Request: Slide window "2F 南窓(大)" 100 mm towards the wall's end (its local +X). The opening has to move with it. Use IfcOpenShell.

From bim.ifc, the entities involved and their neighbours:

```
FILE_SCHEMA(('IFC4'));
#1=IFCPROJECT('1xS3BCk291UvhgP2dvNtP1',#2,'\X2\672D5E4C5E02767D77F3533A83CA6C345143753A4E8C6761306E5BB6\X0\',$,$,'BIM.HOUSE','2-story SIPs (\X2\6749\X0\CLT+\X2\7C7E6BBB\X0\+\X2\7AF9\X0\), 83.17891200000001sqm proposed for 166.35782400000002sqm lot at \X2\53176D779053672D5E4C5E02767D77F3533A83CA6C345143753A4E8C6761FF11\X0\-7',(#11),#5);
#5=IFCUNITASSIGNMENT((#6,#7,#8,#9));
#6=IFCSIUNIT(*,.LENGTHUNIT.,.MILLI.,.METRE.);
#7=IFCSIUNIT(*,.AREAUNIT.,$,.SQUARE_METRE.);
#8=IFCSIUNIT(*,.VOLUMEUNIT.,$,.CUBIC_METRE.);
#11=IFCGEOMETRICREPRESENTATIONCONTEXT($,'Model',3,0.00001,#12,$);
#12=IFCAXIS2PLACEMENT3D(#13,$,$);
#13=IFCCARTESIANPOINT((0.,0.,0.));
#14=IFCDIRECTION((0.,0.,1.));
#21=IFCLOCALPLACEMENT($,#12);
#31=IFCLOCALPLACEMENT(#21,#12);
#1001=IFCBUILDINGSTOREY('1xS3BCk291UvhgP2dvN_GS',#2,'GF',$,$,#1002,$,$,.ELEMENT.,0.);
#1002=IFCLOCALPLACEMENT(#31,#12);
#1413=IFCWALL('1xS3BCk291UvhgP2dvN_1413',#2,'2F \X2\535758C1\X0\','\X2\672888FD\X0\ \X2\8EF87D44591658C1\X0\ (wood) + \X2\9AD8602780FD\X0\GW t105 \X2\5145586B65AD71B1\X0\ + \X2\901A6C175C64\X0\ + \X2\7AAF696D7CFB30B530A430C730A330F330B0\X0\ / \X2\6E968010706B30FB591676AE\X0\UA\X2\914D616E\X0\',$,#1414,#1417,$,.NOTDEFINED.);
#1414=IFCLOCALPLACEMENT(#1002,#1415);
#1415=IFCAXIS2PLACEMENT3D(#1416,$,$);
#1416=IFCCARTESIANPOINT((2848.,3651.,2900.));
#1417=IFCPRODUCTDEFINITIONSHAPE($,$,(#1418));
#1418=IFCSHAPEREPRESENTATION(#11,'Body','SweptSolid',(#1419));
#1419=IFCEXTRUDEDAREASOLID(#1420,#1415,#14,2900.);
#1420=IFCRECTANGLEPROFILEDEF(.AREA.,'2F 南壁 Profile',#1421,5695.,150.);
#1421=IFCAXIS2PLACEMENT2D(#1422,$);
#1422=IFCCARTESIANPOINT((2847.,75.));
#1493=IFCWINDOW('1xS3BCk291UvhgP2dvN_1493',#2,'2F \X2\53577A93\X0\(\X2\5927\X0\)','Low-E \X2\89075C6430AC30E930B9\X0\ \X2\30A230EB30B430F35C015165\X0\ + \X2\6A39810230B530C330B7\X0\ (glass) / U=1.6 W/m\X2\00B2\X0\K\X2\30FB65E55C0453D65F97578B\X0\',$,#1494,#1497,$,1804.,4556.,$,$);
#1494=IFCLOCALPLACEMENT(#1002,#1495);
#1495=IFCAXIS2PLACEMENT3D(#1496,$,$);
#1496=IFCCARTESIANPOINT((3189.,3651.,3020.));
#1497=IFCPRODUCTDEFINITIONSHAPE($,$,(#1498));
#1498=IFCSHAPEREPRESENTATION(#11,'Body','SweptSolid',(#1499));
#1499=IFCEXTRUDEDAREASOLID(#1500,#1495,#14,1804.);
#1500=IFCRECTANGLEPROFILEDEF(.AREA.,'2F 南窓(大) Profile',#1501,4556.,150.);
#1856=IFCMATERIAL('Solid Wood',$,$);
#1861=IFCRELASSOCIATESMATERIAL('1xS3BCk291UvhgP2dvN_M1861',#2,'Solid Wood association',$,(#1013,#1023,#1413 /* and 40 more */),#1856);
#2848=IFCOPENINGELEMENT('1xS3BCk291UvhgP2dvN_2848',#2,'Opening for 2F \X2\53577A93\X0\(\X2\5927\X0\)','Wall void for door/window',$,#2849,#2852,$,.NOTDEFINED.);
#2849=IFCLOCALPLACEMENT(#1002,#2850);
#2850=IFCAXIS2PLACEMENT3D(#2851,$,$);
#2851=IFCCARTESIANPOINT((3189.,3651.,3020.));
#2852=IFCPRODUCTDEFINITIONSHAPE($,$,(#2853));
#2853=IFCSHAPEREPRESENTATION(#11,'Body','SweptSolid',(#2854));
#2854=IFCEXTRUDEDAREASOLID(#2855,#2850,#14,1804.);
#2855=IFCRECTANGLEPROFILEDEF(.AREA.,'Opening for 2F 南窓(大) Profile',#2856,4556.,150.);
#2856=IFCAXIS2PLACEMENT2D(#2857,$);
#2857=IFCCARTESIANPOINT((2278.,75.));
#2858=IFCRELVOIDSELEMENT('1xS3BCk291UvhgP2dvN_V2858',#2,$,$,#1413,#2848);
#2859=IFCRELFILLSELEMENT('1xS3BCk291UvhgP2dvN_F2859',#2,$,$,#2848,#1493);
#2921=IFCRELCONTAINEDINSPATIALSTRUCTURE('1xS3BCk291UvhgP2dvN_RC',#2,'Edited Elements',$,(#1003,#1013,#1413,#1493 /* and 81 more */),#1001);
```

```python
import ifcopenshell
import ifcopenshell.api.geometry
import ifcopenshell.util.placement
import ifcopenshell.util.unit

model = ifcopenshell.open("bim.ifc")
unit_scale = ifcopenshell.util.unit.calculate_unit_scale(model)

window = model.by_guid("1xS3BCk291UvhgP2dvN_1493")
opening = window.FillsVoids[0].RelatingOpeningElement
wall = opening.VoidsElements[0].RelatingBuildingElement

wall_matrix = ifcopenshell.util.placement.get_local_placement(wall.ObjectPlacement)
shift = wall_matrix[:3, 0] * 0.1 / unit_scale
before = ifcopenshell.util.placement.get_local_placement(window.ObjectPlacement)[:3, 3].copy()

# The window is not placed relative to its opening, so move both.
for product in (opening, window):
    matrix = ifcopenshell.util.placement.get_local_placement(product.ObjectPlacement)
    matrix[:3, 3] += shift
    ifcopenshell.api.geometry.edit_object_placement(model, product=product, matrix=matrix, is_si=False)

after = ifcopenshell.util.placement.get_local_placement(window.ObjectPlacement)[:3, 3]
print("window moved by", (after - before).round(3) + 0.0)

model.write("bim_edited.ifc")
```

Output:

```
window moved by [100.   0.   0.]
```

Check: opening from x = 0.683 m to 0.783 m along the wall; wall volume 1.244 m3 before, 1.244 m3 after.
